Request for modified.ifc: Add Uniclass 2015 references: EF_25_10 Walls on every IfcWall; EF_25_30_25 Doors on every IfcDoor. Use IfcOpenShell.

First a look at what the model holds.

```python
import ifcopenshell

model = ifcopenshell.open("modified.ifc")
print(model.schema)
print("classifications:", [c.Name for c in model.by_type("IfcClassification")])
for ifc_class in ("IfcDoor", "IfcRoof", "IfcStair", "IfcWall", "IfcWindow"):
    print(ifc_class, len(model.by_type(ifc_class)))
```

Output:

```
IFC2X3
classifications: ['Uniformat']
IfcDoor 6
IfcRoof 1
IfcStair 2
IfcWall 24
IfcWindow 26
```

```python
import ifcopenshell
import ifcopenshell.api.classification

model = ifcopenshell.open("modified.ifc")

# IFC2X3 requires Source and Edition and has no link from the project to the system.
system = model.create_entity("IfcClassification", Source="NBS", Edition="2015", Name="Uniclass 2015")

codes = {
    "IfcWall": ("EF_25_10", "Walls"),
    "IfcDoor": ("EF_25_30_25", "Doors"),
}
for ifc_class, (code, name) in codes.items():
    products = model.by_type(ifc_class)
    ifcopenshell.api.classification.add_reference(
        model, products=products, classification=system, identification=code, name=name
    )
    print(code, len(products))

model.write("modified_v2.ifc")
```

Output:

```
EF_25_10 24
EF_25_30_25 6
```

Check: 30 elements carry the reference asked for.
